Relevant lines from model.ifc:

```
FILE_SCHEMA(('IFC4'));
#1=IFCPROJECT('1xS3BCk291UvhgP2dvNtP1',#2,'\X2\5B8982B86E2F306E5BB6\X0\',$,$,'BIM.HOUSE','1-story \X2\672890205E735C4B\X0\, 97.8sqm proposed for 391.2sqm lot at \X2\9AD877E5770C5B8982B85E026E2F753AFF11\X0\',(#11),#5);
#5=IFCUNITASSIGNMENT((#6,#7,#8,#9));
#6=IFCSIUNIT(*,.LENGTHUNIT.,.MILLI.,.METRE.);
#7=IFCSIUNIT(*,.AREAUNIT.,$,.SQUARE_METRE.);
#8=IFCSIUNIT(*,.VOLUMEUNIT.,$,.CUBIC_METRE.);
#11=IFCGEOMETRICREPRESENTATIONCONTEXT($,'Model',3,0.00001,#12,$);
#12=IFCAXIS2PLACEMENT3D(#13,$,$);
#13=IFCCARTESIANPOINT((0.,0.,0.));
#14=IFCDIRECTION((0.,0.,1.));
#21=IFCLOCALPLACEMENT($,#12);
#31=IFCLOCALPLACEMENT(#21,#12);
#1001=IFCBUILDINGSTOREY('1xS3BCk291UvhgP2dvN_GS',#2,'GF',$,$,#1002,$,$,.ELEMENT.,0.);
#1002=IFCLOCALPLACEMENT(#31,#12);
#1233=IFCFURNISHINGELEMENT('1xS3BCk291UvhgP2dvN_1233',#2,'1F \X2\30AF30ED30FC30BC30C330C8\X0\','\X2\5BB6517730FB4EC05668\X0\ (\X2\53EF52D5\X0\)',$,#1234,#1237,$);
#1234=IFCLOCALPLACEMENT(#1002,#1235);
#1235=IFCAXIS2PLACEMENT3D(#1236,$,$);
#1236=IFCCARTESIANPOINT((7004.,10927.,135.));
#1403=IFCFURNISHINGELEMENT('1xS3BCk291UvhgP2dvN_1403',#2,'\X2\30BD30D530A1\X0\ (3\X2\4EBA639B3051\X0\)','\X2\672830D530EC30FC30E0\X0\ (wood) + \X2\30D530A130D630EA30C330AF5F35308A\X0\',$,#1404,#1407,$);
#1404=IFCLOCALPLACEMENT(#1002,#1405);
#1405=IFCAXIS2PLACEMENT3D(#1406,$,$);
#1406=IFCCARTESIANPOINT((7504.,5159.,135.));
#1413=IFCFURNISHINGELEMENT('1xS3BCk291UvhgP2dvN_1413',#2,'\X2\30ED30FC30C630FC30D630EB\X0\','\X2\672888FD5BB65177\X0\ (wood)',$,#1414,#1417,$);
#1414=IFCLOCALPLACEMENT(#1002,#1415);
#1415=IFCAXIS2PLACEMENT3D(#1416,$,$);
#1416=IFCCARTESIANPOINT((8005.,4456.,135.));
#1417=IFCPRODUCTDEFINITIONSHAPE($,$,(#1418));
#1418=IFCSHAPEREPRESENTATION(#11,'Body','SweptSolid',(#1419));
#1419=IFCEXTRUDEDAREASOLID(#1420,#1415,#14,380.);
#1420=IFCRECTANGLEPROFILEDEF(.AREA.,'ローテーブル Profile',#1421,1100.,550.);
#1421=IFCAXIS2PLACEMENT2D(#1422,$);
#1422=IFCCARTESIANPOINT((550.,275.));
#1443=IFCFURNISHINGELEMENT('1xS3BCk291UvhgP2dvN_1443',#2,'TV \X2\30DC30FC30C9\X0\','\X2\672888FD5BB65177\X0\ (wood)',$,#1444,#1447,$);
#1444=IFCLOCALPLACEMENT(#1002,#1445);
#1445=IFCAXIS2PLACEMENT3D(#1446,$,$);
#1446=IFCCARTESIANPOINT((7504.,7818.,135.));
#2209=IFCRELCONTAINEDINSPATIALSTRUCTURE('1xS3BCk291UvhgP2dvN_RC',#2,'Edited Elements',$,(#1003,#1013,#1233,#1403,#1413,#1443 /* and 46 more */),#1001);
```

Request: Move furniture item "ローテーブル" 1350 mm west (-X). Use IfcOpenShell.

```python
import ifcopenshell
import ifcopenshell.api.geometry
import ifcopenshell.util.placement
import ifcopenshell.util.unit

model = ifcopenshell.open("model.ifc")
unit_scale = ifcopenshell.util.unit.calculate_unit_scale(model)

item = model.by_guid("1xS3BCk291UvhgP2dvN_1413")
matrix = ifcopenshell.util.placement.get_local_placement(item.ObjectPlacement)
matrix[0, 3] -= 1.35 / unit_scale
ifcopenshell.api.geometry.edit_object_placement(model, product=item, matrix=matrix, is_si=False)

print(ifcopenshell.util.placement.get_local_placement(item.ObjectPlacement).round(3) + 0.0)

model.write("model_rev.ifc")
```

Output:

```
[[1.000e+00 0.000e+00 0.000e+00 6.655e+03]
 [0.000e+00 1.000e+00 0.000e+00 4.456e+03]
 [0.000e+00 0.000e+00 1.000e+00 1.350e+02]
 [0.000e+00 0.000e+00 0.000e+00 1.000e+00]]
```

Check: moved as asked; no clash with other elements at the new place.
